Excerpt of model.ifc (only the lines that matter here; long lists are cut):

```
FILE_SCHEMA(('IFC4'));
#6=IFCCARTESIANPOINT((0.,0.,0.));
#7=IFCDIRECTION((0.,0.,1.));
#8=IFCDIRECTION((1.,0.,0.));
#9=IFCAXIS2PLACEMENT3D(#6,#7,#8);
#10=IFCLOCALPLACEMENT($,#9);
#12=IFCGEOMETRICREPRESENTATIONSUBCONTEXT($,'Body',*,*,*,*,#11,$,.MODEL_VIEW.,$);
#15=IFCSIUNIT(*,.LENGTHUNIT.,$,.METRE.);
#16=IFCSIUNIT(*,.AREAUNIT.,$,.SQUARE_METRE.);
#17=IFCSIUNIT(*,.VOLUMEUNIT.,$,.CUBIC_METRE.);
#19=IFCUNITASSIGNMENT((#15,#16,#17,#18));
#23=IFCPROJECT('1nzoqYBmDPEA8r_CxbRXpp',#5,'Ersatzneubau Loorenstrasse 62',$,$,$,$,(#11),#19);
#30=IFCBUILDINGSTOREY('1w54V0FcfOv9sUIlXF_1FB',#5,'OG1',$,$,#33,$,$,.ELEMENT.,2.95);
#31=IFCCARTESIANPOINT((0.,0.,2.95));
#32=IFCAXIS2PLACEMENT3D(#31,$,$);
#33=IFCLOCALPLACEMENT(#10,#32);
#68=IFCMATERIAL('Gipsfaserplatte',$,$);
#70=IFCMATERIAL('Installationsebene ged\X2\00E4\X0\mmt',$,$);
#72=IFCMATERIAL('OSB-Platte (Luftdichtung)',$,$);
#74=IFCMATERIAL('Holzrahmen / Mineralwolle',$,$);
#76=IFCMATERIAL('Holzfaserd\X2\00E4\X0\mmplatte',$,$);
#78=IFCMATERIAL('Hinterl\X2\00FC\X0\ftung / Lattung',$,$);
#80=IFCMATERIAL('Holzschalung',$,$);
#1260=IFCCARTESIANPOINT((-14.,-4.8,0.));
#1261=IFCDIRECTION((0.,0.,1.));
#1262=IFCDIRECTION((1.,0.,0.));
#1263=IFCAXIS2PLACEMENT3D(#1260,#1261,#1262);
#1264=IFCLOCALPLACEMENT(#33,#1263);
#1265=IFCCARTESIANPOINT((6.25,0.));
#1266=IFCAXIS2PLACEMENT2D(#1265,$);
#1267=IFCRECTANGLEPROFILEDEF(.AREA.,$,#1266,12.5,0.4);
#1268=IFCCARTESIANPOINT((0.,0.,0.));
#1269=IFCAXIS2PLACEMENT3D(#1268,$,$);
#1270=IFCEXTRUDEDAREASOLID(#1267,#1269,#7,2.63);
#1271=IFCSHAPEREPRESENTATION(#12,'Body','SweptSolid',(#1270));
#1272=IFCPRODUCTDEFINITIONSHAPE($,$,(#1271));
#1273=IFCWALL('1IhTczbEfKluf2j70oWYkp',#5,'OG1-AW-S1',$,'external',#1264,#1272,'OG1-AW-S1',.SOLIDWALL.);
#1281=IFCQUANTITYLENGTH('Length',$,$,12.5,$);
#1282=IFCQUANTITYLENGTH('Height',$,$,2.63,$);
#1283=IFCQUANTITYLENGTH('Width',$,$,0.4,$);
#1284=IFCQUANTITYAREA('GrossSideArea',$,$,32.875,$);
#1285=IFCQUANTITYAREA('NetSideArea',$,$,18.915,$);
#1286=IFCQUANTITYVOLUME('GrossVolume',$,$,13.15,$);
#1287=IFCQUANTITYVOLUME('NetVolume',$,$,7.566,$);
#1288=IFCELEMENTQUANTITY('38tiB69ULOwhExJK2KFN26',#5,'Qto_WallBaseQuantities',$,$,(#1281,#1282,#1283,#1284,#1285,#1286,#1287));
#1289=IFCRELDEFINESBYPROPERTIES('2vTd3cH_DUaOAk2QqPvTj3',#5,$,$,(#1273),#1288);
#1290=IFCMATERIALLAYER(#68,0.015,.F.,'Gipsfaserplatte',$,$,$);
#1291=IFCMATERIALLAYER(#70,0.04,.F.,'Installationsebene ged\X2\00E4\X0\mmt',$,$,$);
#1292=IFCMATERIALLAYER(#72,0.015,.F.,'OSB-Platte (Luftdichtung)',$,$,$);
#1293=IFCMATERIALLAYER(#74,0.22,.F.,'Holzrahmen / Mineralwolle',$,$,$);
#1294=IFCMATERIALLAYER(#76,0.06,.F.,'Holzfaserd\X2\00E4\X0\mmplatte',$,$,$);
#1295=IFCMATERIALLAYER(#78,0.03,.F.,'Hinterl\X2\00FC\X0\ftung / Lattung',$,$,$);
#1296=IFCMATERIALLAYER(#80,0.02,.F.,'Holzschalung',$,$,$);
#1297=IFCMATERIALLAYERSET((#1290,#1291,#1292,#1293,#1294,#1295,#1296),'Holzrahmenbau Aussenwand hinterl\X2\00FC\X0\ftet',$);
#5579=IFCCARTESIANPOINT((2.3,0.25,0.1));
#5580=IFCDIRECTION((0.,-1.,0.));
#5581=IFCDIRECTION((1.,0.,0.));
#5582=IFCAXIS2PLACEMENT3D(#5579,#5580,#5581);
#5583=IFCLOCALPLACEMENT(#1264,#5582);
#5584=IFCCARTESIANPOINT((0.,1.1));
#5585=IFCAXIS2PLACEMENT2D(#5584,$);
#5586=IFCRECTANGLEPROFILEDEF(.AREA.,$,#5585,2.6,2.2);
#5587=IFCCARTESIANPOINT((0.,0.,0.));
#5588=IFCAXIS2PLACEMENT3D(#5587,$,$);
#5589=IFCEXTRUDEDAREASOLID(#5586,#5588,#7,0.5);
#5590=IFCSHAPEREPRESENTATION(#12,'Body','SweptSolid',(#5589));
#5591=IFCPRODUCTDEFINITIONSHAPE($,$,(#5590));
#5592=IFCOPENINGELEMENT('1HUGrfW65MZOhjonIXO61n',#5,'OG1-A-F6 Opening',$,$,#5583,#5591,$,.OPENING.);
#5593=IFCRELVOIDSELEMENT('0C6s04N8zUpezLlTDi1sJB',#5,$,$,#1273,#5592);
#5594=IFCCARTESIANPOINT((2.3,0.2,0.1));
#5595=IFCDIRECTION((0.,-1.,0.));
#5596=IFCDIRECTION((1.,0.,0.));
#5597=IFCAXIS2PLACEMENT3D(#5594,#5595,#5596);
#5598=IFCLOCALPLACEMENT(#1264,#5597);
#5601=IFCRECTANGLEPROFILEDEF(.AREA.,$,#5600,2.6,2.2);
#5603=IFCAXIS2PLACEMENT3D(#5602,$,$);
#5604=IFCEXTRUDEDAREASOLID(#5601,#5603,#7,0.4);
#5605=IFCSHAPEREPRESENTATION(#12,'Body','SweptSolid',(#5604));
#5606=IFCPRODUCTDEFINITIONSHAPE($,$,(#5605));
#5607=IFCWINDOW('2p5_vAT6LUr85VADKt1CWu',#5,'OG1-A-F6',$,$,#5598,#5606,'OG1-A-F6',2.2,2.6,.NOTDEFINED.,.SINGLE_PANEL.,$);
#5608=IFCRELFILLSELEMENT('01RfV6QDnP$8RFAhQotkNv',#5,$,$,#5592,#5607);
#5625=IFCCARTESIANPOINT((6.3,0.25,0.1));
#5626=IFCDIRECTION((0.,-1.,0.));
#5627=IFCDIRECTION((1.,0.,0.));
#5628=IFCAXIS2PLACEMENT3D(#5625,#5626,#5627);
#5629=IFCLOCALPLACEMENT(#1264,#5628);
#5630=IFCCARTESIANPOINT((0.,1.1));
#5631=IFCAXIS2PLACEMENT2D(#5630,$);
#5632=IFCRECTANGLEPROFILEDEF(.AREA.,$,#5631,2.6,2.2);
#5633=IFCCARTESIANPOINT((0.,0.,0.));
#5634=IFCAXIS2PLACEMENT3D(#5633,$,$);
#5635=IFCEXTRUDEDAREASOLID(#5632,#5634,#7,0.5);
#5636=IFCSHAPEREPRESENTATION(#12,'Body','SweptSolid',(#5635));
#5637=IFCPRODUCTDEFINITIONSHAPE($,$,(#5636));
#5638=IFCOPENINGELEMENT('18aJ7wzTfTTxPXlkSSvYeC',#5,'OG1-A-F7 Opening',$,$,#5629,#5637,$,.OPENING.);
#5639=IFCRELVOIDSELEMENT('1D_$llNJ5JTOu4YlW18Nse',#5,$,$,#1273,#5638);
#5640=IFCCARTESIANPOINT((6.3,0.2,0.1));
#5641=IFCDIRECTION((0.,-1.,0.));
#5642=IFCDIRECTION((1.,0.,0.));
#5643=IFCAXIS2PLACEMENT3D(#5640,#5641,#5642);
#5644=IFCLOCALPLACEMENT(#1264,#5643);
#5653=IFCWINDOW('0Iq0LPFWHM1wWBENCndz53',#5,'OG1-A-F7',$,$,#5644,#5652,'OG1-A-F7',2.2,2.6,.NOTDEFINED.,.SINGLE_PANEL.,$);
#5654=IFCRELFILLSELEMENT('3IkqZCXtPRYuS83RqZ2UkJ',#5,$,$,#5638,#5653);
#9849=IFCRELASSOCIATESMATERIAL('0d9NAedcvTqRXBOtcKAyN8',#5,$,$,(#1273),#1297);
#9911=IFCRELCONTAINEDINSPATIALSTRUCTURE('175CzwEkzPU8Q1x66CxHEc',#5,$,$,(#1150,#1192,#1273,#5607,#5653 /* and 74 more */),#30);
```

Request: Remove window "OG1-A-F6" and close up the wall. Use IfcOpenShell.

```python
import ifcopenshell
import ifcopenshell.api.feature
import ifcopenshell.api.pset
import ifcopenshell.api.root
import ifcopenshell.geom
import ifcopenshell.util.element
import ifcopenshell.util.shape
import ifcopenshell.util.unit

model = ifcopenshell.open("model.ifc")
area_scale = ifcopenshell.util.unit.calculate_unit_scale(model, "AREAUNIT")
volume_scale = ifcopenshell.util.unit.calculate_unit_scale(model, "VOLUMEUNIT")
settings = ifcopenshell.geom.settings()


def volume(element):
    """Net volume in cubic metres, openings subtracted."""
    shape = ifcopenshell.geom.create_shape(settings, element)
    return ifcopenshell.util.shape.get_volume(shape.geometry)


window = model.by_guid("2p5_vAT6LUr85VADKt1CWu")
opening = window.FillsVoids[0].RelatingOpeningElement
wall = opening.VoidsElements[0].RelatingBuildingElement
before = volume(wall)

ifcopenshell.api.root.remove_product(model, product=window)
ifcopenshell.api.feature.remove_feature(model, feature=opening)

after = volume(wall)
thickness = 0.4  # wall thickness in metres

# Update the wall's stored quantities.
qto = model.by_id(ifcopenshell.util.element.get_pset(wall, "Qto_WallBaseQuantities", should_inherit=False)["id"])
ifcopenshell.api.pset.edit_qto(model, qto=qto, properties={
    "NetSideArea": after / thickness / area_scale,
    "NetVolume": after / volume_scale,
})

print(f"wall volume {before:.3f} -> {after:.3f} m3")

model.write("model-out.ifc")
```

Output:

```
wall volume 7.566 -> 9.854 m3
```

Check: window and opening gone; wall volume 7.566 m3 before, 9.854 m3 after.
